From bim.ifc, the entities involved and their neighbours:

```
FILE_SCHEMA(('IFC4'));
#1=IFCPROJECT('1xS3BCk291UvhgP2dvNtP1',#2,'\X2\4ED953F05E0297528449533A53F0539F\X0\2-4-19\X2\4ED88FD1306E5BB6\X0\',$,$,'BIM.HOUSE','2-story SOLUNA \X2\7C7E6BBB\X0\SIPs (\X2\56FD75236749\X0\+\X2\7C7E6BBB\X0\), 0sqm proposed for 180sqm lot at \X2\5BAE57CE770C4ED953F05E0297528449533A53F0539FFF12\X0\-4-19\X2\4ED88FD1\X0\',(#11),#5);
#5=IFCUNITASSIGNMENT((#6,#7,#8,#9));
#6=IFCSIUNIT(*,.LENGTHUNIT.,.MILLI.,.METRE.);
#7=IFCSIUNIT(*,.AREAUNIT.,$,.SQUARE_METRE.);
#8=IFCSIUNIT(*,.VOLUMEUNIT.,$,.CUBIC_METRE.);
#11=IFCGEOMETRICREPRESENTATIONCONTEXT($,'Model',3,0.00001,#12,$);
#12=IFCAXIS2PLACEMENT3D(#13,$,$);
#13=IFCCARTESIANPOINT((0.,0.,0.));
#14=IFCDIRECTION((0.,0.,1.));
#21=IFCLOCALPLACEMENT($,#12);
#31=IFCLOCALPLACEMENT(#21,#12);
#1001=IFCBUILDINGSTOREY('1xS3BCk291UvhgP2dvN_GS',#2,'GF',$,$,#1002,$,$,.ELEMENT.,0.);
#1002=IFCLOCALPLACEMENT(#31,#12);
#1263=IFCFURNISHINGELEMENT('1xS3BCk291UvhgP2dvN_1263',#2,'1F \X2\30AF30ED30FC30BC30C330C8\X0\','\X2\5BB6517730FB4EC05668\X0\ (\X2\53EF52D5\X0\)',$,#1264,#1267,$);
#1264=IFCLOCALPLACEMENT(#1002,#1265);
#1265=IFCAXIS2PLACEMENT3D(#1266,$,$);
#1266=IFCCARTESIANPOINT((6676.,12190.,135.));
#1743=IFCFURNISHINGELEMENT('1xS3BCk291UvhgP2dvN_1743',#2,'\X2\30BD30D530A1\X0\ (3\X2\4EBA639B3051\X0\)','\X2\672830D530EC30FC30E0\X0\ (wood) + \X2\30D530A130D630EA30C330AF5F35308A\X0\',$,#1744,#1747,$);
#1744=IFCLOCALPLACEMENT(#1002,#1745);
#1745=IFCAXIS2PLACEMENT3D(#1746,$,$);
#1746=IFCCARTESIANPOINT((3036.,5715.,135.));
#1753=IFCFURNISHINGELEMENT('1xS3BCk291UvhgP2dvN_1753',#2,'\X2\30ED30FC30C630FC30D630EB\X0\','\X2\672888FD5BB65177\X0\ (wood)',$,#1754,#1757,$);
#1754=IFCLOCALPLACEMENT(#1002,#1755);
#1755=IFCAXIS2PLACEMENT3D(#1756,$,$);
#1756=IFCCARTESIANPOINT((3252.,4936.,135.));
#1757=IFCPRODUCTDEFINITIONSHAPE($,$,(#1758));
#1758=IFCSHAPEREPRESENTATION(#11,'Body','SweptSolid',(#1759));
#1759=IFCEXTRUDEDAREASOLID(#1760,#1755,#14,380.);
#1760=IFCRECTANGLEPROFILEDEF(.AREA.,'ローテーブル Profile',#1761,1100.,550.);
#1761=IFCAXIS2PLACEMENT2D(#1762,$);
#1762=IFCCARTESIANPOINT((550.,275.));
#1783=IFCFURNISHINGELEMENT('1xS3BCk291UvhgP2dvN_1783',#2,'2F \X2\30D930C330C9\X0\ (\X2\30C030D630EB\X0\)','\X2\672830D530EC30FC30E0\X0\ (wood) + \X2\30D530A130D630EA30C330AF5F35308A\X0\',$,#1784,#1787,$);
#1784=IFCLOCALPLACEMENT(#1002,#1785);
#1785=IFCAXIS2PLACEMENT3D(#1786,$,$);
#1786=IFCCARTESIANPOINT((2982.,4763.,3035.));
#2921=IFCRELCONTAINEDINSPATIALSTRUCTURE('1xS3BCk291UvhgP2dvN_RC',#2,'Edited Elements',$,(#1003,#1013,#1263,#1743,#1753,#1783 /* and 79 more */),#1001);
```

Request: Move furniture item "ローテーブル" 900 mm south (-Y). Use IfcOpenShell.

```python
import ifcopenshell
import ifcopenshell.api.geometry
import ifcopenshell.util.placement
import ifcopenshell.util.unit

model = ifcopenshell.open("bim.ifc")
unit_scale = ifcopenshell.util.unit.calculate_unit_scale(model)

item = model.by_guid("1xS3BCk291UvhgP2dvN_1753")
matrix = ifcopenshell.util.placement.get_local_placement(item.ObjectPlacement)
matrix[1, 3] -= 0.9 / unit_scale
ifcopenshell.api.geometry.edit_object_placement(model, product=item, matrix=matrix, is_si=False)

print(ifcopenshell.util.placement.get_local_placement(item.ObjectPlacement).round(3) + 0.0)

model.write("bim_v2.ifc")
```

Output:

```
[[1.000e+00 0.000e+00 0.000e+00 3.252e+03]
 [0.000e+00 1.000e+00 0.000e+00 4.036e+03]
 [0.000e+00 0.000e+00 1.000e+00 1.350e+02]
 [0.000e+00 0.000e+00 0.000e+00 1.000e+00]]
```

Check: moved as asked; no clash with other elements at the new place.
